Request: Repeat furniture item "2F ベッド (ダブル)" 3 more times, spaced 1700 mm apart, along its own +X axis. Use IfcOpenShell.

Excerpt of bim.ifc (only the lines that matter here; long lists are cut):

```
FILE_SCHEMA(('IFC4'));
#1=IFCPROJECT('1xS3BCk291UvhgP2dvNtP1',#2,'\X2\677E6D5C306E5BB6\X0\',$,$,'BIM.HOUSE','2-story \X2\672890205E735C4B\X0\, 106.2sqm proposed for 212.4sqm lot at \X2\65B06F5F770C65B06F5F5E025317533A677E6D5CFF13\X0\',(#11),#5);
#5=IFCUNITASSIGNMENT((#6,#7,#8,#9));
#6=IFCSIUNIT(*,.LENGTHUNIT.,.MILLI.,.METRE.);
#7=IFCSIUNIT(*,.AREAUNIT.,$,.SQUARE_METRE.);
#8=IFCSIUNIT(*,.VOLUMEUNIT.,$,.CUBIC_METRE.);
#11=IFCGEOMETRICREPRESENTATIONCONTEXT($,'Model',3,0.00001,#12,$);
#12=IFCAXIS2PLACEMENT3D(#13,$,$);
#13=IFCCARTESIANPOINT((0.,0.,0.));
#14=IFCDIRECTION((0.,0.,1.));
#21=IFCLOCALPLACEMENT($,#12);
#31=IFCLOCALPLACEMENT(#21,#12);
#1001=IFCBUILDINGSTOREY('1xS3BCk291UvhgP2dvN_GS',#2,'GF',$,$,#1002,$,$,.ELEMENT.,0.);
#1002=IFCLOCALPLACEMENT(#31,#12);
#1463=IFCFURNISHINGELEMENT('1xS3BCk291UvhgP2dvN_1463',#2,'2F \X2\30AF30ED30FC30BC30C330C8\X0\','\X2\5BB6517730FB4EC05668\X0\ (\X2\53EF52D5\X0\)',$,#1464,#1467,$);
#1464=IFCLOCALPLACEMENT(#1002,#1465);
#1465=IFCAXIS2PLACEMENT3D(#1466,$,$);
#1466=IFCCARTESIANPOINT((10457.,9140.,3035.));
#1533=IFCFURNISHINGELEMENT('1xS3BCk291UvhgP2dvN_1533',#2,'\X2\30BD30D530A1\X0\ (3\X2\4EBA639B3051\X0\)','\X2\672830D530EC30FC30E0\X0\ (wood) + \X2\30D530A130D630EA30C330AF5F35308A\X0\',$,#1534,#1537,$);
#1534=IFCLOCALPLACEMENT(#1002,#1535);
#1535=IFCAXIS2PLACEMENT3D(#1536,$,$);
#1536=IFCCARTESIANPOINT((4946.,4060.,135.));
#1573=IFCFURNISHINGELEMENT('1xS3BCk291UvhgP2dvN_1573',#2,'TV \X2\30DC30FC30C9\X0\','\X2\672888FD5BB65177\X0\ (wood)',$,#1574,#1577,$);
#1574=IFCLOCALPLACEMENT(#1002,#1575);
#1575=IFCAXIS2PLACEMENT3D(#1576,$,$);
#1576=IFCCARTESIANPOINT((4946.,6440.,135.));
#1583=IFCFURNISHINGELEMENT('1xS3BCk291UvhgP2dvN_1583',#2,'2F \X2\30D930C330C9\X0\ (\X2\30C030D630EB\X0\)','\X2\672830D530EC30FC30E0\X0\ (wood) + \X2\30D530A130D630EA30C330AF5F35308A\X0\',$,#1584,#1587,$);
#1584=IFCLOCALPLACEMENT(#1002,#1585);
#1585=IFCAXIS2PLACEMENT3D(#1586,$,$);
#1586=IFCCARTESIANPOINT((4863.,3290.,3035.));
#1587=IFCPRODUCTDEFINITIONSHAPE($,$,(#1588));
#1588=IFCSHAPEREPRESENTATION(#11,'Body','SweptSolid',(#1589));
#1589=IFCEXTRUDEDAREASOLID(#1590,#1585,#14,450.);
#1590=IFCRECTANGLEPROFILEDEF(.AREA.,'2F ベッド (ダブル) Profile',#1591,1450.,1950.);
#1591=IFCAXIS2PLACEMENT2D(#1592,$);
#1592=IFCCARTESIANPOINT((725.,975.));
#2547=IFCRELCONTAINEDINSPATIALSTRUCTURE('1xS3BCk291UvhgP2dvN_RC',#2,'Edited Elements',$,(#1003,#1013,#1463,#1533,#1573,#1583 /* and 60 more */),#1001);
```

```python
import ifcopenshell
import ifcopenshell.api.geometry
import ifcopenshell.api.root
import ifcopenshell.util.element
import ifcopenshell.util.placement
import ifcopenshell.util.unit

model = ifcopenshell.open("bim.ifc")
unit_scale = ifcopenshell.util.unit.calculate_unit_scale(model)


def reuse_history(source, copy):
    """copy_class also copies each property set's owner history, people and application; keep the originals."""
    for rel in copy.IsDefinedBy:
        if rel.is_a("IfcRelDefinesByProperties") and (history := rel.RelatingPropertyDefinition.OwnerHistory):
            rel.RelatingPropertyDefinition.OwnerHistory = source.OwnerHistory
            ifcopenshell.util.element.remove_deep2(model, history)


source = model.by_id(1583)
base = ifcopenshell.util.placement.get_local_placement(source.ObjectPlacement)
step = base[:3, 0] * 1.7 / unit_scale

for i in range(1, 4):
    copy = ifcopenshell.api.root.copy_class(model, product=source)
    copy.Representation = ifcopenshell.util.element.copy_deep(
        model, source.Representation, exclude=["IfcGeometricRepresentationContext", "IfcRepresentationMap"]
    )
    reuse_history(source, copy)
    matrix = base.copy()
    matrix[:3, 3] += i * step
    print("added at", matrix[:3, 3].round(3) + 0.0)
    ifcopenshell.api.geometry.edit_object_placement(model, product=copy, matrix=matrix, is_si=False)

model.write("bim_edited.ifc")
```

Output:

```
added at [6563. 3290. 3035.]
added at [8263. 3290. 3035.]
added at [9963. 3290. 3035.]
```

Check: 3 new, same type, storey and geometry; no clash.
